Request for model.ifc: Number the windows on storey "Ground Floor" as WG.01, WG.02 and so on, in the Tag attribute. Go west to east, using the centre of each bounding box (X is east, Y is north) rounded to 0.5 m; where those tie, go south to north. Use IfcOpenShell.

First a look at what the model holds.

```python
import ifcopenshell
import ifcopenshell.util.element
import ifcopenshell.util.placement

model = ifcopenshell.open("model.ifc")
print(model.schema)
storey = next(s for s in model.by_type("IfcBuildingStorey") if s.Name == "Ground Floor")
windows = [e for e in ifcopenshell.util.element.get_decomposition(storey) if e.is_a("IfcWindow")]
for e in sorted(windows, key=lambda e: e.id()):
    origin = ifcopenshell.util.placement.get_local_placement(e.ObjectPlacement)[:3, 3]
    print(e.id(), e.Tag, e.Name, origin.round(2) + 0.0, sep=" | ")
```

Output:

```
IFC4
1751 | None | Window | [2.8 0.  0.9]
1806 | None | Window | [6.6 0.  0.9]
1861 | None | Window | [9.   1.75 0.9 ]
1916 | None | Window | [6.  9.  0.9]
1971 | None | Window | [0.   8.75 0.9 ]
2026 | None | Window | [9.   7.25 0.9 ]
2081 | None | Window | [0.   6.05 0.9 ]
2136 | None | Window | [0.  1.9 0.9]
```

```python
import ifcopenshell
import ifcopenshell.geom
import ifcopenshell.util.element
import ifcopenshell.util.shape

model = ifcopenshell.open("model.ifc")
settings = ifcopenshell.geom.settings()
settings.set("use-world-coords", True)


def centre(element):
    shape = ifcopenshell.geom.create_shape(settings, element)
    return ifcopenshell.util.shape.get_bbox_centroid(shape.geometry)


storey = next(s for s in model.by_type("IfcBuildingStorey") if s.Name == "Ground Floor")
windows = [e for e in ifcopenshell.util.element.get_decomposition(storey) if e.is_a("IfcWindow")]

# Insertion points can sit at a corner or the storey origin, so sort by the geometry (in metres).
centres = {e: centre(e) for e in windows}
windows.sort(key=lambda e: (round(centres[e][0] / 0.5), centres[e][1]))

for i, e in enumerate(windows, start=1):
    number = f"WG.{i:02d}"
    e.Tag = number
    print(e.id(), number)

model.write("model-out.ifc")
```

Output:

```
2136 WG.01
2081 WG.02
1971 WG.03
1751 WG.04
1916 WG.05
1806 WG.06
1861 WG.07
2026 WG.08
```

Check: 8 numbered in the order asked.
